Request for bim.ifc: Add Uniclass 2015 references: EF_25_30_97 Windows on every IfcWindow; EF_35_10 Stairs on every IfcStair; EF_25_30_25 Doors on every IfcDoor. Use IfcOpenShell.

First a look at what the model holds.

```python
import ifcopenshell

model = ifcopenshell.open("bim.ifc")
print(model.schema)
print("classifications:", [c.Name for c in model.by_type("IfcClassification")])
for ifc_class in ("IfcDoor", "IfcRoof", "IfcStair", "IfcWall", "IfcWindow"):
    print(ifc_class, len(model.by_type(ifc_class)))
```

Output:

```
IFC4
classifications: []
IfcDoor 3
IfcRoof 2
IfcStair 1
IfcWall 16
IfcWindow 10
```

```python
import ifcopenshell
import ifcopenshell.api.classification

model = ifcopenshell.open("bim.ifc")

system = ifcopenshell.api.classification.add_classification(model, classification="Uniclass 2015")

codes = {
    "IfcWindow": ("EF_25_30_97", "Windows"),
    "IfcStair": ("EF_35_10", "Stairs"),
    "IfcDoor": ("EF_25_30_25", "Doors"),
}
for ifc_class, (code, name) in codes.items():
    products = model.by_type(ifc_class)
    ifcopenshell.api.classification.add_reference(
        model, products=products, classification=system, identification=code, name=name
    )
    print(code, len(products))

model.write("bim_updated.ifc")
```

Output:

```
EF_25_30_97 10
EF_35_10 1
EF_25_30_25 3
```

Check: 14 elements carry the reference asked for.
